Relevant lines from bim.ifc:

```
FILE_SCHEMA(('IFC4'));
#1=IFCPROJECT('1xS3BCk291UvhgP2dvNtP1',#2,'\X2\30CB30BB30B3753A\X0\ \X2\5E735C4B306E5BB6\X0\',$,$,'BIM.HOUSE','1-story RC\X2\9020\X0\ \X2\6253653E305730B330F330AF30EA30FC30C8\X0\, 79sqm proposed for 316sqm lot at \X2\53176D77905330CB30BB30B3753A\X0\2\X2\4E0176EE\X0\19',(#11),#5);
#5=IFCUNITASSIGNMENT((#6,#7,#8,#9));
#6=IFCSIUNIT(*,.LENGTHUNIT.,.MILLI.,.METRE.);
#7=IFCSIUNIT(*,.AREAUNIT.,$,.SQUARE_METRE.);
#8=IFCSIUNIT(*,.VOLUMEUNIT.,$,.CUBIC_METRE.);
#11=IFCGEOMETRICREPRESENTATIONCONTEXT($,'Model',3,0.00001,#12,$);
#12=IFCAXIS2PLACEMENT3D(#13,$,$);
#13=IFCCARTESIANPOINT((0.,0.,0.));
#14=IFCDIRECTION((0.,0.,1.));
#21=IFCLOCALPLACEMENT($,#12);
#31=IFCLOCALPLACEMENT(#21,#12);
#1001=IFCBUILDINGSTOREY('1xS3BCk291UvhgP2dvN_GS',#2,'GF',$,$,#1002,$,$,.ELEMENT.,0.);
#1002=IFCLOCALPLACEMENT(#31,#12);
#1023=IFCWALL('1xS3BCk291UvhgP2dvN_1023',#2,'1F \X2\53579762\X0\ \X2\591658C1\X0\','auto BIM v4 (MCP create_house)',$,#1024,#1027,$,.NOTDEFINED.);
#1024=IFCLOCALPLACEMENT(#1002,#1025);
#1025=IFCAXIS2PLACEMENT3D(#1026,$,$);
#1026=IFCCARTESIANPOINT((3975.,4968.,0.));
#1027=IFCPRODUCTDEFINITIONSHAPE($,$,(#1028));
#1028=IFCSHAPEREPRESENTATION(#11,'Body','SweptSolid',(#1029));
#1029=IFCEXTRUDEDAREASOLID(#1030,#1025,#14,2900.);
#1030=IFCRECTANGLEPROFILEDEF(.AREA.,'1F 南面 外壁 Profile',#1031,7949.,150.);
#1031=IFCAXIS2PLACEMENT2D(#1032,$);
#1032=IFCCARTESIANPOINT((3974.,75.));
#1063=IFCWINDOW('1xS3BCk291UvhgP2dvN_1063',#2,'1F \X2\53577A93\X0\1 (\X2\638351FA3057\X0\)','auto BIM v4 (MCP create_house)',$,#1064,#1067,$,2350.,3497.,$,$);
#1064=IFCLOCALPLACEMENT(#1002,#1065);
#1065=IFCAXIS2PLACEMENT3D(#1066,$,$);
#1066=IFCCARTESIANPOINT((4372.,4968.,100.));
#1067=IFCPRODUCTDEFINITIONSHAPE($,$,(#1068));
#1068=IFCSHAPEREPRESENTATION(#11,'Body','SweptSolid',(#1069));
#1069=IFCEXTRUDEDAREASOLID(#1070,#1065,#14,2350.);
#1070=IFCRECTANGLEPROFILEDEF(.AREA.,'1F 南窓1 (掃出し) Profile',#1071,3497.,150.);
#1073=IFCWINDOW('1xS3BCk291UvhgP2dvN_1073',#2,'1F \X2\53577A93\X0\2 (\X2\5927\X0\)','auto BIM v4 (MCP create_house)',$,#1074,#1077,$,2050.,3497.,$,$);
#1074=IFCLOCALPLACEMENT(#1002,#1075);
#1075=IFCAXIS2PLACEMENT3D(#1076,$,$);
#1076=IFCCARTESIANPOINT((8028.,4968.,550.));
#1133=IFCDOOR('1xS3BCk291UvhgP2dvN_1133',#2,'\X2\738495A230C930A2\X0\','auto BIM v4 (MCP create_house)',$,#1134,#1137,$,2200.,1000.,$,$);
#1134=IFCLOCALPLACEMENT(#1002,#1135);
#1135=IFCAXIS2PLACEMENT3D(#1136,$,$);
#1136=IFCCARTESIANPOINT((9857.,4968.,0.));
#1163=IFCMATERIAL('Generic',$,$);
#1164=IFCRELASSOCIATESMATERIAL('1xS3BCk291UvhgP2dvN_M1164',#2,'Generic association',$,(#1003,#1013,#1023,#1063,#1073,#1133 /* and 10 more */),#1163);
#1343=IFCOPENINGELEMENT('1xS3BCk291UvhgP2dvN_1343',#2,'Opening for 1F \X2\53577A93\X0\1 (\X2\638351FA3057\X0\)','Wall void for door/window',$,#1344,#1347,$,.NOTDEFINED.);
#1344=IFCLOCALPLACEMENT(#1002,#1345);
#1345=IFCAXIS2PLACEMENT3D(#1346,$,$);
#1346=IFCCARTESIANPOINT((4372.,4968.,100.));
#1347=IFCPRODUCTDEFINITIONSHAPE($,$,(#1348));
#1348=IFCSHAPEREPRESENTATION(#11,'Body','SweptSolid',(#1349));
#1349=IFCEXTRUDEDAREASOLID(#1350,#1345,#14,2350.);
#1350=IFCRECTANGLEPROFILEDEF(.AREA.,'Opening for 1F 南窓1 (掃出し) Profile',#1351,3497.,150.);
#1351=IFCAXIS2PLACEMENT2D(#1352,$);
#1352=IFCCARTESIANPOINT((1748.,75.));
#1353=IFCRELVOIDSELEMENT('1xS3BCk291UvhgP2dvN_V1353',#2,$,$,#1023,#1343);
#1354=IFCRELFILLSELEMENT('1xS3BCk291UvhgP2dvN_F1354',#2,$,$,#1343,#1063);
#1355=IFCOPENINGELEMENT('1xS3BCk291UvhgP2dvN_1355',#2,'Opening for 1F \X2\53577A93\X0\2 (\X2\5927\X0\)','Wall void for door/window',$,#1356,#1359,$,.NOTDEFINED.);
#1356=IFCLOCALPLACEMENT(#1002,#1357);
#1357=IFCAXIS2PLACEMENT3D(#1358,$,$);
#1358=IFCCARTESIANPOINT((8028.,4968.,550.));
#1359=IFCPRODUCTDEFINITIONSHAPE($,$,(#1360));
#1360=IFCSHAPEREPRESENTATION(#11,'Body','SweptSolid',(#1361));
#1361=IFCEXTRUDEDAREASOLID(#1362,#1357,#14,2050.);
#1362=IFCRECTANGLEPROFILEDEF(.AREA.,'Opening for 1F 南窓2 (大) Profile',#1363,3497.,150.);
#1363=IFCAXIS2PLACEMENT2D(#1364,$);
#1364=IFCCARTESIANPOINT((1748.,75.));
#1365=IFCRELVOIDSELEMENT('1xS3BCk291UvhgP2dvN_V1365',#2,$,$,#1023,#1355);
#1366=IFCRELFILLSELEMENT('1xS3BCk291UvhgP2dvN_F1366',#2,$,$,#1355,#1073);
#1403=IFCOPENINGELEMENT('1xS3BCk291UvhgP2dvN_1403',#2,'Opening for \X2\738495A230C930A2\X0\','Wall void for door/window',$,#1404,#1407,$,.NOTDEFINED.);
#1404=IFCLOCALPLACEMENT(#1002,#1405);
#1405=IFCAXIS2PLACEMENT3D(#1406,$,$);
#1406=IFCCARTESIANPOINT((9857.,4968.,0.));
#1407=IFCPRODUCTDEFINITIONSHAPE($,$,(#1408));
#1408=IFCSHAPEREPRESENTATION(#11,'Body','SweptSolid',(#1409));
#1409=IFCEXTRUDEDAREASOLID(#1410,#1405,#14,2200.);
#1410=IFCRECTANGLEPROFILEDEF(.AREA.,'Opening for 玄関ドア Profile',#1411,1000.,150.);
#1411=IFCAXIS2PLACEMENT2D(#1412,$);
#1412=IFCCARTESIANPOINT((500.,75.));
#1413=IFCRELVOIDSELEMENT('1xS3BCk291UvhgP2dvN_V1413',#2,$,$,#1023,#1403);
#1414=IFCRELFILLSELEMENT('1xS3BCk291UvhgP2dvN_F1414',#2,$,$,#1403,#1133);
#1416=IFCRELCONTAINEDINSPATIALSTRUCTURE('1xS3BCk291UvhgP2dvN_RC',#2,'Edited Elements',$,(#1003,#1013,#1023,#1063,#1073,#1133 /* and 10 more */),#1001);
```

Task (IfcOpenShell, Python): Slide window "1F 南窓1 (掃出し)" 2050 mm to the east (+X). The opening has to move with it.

```python
import ifcopenshell
import ifcopenshell.api.geometry
import ifcopenshell.util.placement

model = ifcopenshell.open("bim.ifc")

window = model.by_guid("1xS3BCk291UvhgP2dvN_1063")
opening = window.FillsVoids[0].RelatingOpeningElement
wall = opening.VoidsElements[0].RelatingBuildingElement

wall_matrix = ifcopenshell.util.placement.get_local_placement(wall.ObjectPlacement)
shift = wall_matrix[:3, 0] * 2050.0
before = ifcopenshell.util.placement.get_local_placement(window.ObjectPlacement)[:3, 3].copy()

# The window is not placed relative to its opening, so move both.
for product in (opening, window):
    matrix = ifcopenshell.util.placement.get_local_placement(product.ObjectPlacement)
    matrix[:3, 3] += shift
    ifcopenshell.api.geometry.edit_object_placement(model, product=product, matrix=matrix, is_si=False)

after = ifcopenshell.util.placement.get_local_placement(window.ObjectPlacement)[:3, 3]
print("window moved by", (after - before).round(3) + 0.0)

model.write("bim_updated.ifc")
```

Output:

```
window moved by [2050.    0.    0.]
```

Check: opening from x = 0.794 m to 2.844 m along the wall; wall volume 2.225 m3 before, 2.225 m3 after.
